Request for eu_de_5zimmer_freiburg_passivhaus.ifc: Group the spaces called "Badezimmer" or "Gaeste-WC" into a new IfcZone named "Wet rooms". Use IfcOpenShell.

First a look at what the model holds.

```python
import ifcopenshell

model = ifcopenshell.open("eu_de_5zimmer_freiburg_passivhaus.ifc")
print(model.schema)
seen = {}
for space in model.by_type("IfcSpace"):
    seen[space.LongName] = seen.get(space.LongName, 0) + 1
for name, count in sorted(seen.items(), key=str):
    print(count, "x", name)
print("zones:", [z.Name for z in model.by_type("IfcZone")][:20])
```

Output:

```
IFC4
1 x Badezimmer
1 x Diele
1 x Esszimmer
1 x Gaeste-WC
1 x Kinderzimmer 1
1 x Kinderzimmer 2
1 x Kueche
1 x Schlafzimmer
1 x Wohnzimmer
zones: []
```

```python
import ifcopenshell
import ifcopenshell.api.group
import ifcopenshell.api.root

model = ifcopenshell.open("eu_de_5zimmer_freiburg_passivhaus.ifc")

names = {"Badezimmer", "Gaeste-WC"}
spaces = [s for s in model.by_type("IfcSpace") if s.LongName in names]

zone = ifcopenshell.api.root.create_entity(model, ifc_class="IfcZone", name="Wet rooms")
ifcopenshell.api.group.assign_group(model, products=spaces, group=zone)
print(len(spaces), "spaces in", zone.Name)

model.write("eu_de_5zimmer_freiburg_passivhaus_v2.ifc")
```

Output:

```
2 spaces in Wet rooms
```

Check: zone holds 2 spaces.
